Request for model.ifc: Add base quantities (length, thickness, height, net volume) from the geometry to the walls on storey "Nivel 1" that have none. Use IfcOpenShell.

First a look at what the model holds.

```python
import ifcopenshell
import ifcopenshell.util.element
import ifcopenshell.util.unit

model = ifcopenshell.open("model.ifc")
print(model.schema)
for unit_type in ("LENGTHUNIT", "AREAUNIT", "VOLUMEUNIT"):
    print(unit_type, ifcopenshell.util.unit.calculate_unit_scale(model, unit_type))
storey = next(s for s in model.by_type("IfcBuildingStorey") if s.Name == "Nivel 1")
walls = [e for e in ifcopenshell.util.element.get_decomposition(storey) if e.is_a("IfcWall")]
for e in sorted(walls, key=lambda e: e.id()):
    print(e.id(), e.is_a(), e.Name, list(ifcopenshell.util.element.get_psets(e, qtos_only=True)), sep=" | ")
```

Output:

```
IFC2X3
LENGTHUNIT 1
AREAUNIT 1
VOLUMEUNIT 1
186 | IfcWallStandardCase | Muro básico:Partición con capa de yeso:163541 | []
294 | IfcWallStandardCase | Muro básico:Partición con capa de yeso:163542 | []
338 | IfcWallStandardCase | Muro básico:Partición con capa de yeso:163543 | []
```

```python
import ifcopenshell
import ifcopenshell.api.pset
import ifcopenshell.geom
import ifcopenshell.util.element
import ifcopenshell.util.shape
import ifcopenshell.util.unit

model = ifcopenshell.open("model.ifc")
unit_scale = ifcopenshell.util.unit.calculate_unit_scale(model)
volume_scale = ifcopenshell.util.unit.calculate_unit_scale(model, "VOLUMEUNIT")
settings = ifcopenshell.geom.settings()

storey = next(s for s in model.by_type("IfcBuildingStorey") if s.Name == "Nivel 1")
walls = [e for e in ifcopenshell.util.element.get_decomposition(storey) if e.is_a("IfcWall")]

for e in sorted(walls, key=lambda e: e.id()):
    if ifcopenshell.util.element.get_psets(e, qtos_only=True, should_inherit=False):
        continue
    # Geometry comes back in metres, in the element's own axes.
    shape = ifcopenshell.geom.create_shape(settings, e)
    values = {
        "Length": ifcopenshell.util.shape.get_x(shape.geometry) / unit_scale,
        "Width": ifcopenshell.util.shape.get_y(shape.geometry) / unit_scale,
        "Height": ifcopenshell.util.shape.get_z(shape.geometry) / unit_scale,
        "NetVolume": ifcopenshell.util.shape.get_volume(shape.geometry) / volume_scale,
    }
    qto = ifcopenshell.api.pset.add_qto(model, product=e, name="BaseQuantities")
    ifcopenshell.api.pset.edit_qto(model, qto=qto, properties=values)
    print(e.id(), {k: round(v, 3) for k, v in values.items()})

model.write("model_edited.ifc")
```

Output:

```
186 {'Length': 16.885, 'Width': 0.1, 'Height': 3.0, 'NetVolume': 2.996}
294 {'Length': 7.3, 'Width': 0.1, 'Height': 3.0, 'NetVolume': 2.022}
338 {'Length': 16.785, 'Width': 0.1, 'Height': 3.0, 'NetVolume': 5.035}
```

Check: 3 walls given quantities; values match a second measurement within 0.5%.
